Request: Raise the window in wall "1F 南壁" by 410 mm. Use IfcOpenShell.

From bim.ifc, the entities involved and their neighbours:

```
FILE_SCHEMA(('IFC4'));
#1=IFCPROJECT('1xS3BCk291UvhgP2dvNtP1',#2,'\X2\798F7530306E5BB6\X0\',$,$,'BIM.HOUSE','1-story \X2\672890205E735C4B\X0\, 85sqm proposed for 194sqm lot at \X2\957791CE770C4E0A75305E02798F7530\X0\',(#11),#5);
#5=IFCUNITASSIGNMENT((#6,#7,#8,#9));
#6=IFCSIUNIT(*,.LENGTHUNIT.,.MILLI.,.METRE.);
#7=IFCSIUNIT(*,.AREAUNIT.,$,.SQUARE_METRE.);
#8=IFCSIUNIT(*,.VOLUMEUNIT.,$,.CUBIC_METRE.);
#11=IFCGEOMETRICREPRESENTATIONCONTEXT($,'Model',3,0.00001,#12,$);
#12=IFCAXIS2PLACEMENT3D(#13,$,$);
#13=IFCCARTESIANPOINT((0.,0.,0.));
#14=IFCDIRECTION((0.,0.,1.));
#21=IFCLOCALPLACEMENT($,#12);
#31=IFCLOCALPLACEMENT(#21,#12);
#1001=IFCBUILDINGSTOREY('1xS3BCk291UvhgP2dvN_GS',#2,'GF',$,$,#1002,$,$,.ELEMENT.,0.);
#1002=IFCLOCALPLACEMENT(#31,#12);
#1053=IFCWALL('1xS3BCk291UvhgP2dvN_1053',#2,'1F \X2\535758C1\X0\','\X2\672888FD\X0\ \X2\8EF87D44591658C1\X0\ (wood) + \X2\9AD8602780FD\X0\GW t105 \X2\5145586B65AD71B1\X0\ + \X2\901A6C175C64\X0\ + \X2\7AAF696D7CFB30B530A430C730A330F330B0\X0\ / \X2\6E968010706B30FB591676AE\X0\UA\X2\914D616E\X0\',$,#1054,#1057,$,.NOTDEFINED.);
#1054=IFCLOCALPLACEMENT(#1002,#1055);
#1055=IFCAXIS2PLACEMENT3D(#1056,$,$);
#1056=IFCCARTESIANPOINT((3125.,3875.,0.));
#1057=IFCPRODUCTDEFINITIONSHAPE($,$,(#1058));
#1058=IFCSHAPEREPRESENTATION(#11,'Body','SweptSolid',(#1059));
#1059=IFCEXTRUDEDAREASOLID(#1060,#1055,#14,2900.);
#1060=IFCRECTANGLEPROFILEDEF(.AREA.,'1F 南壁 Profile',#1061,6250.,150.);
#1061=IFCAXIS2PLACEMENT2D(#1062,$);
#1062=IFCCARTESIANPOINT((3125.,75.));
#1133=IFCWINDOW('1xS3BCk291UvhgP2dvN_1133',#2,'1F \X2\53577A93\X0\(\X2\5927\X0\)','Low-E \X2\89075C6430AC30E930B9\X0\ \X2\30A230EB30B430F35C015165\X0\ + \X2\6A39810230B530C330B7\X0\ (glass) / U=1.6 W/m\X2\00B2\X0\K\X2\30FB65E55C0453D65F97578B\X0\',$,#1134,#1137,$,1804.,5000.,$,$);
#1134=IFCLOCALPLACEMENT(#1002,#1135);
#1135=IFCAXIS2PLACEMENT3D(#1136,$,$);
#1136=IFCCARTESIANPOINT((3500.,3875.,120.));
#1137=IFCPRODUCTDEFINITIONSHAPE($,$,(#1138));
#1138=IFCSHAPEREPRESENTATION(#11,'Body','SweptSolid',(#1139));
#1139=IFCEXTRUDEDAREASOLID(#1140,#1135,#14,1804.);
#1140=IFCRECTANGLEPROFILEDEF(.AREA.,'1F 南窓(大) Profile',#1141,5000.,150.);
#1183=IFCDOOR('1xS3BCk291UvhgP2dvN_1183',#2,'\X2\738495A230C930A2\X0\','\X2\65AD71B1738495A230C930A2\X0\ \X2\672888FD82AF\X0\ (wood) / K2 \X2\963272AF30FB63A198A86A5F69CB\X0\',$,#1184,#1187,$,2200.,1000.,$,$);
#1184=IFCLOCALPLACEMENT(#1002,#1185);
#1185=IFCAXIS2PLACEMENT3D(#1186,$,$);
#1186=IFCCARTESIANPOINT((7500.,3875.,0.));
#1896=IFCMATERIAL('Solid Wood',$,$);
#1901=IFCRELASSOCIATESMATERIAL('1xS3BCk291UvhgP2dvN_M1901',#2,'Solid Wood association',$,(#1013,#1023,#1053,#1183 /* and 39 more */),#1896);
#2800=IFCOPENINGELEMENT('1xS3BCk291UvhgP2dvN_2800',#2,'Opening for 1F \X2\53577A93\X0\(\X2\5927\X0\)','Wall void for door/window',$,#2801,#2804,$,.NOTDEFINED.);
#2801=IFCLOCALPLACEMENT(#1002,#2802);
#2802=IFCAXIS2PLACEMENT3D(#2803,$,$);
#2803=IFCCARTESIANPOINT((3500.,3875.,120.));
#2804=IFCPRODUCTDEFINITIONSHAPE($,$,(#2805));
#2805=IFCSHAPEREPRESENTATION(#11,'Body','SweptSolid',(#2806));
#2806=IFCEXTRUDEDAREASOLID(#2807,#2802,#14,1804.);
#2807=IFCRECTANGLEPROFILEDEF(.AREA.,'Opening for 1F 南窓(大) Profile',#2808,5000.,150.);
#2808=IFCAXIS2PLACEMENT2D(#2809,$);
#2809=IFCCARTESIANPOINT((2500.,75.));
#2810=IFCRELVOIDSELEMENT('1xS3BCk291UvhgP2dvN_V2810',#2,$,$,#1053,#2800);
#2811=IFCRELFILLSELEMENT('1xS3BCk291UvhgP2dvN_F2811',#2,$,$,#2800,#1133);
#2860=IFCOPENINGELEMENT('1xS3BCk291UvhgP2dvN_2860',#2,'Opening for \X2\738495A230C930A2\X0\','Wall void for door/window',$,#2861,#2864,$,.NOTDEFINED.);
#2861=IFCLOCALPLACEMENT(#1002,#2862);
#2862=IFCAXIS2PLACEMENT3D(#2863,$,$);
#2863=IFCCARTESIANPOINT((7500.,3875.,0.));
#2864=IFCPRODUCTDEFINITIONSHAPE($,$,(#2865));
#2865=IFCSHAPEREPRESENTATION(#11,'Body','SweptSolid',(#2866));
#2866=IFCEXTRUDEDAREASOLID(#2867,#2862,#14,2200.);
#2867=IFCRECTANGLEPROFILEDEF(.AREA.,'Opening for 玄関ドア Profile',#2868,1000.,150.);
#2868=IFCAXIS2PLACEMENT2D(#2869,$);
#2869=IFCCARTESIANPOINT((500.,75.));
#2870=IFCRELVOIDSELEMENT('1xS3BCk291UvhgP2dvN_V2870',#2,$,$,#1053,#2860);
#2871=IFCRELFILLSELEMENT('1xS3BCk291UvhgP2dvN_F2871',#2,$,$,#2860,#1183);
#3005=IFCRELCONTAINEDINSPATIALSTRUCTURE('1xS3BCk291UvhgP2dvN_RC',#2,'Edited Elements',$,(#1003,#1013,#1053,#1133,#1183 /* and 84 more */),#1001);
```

```python
import numpy as np
import ifcopenshell
import ifcopenshell.api.geometry
import ifcopenshell.util.placement
import ifcopenshell.util.unit

model = ifcopenshell.open("bim.ifc")
unit_scale = ifcopenshell.util.unit.calculate_unit_scale(model)

window = model.by_guid("1xS3BCk291UvhgP2dvN_1133")
opening = window.FillsVoids[0].RelatingOpeningElement
dz = 0.41 / unit_scale

shift = np.array([0.0, 0.0, dz])
# The window is not placed relative to its opening, so move both.
for product in (opening, window):
    matrix = ifcopenshell.util.placement.get_local_placement(product.ObjectPlacement)
    matrix[:3, 3] += shift
    ifcopenshell.api.geometry.edit_object_placement(model, product=product, matrix=matrix, is_si=False)

print(f"moved by {dz * unit_scale:+.3f} m")

model.write("bim_edited.ifc")
```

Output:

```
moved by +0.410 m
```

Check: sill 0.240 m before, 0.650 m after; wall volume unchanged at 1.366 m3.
